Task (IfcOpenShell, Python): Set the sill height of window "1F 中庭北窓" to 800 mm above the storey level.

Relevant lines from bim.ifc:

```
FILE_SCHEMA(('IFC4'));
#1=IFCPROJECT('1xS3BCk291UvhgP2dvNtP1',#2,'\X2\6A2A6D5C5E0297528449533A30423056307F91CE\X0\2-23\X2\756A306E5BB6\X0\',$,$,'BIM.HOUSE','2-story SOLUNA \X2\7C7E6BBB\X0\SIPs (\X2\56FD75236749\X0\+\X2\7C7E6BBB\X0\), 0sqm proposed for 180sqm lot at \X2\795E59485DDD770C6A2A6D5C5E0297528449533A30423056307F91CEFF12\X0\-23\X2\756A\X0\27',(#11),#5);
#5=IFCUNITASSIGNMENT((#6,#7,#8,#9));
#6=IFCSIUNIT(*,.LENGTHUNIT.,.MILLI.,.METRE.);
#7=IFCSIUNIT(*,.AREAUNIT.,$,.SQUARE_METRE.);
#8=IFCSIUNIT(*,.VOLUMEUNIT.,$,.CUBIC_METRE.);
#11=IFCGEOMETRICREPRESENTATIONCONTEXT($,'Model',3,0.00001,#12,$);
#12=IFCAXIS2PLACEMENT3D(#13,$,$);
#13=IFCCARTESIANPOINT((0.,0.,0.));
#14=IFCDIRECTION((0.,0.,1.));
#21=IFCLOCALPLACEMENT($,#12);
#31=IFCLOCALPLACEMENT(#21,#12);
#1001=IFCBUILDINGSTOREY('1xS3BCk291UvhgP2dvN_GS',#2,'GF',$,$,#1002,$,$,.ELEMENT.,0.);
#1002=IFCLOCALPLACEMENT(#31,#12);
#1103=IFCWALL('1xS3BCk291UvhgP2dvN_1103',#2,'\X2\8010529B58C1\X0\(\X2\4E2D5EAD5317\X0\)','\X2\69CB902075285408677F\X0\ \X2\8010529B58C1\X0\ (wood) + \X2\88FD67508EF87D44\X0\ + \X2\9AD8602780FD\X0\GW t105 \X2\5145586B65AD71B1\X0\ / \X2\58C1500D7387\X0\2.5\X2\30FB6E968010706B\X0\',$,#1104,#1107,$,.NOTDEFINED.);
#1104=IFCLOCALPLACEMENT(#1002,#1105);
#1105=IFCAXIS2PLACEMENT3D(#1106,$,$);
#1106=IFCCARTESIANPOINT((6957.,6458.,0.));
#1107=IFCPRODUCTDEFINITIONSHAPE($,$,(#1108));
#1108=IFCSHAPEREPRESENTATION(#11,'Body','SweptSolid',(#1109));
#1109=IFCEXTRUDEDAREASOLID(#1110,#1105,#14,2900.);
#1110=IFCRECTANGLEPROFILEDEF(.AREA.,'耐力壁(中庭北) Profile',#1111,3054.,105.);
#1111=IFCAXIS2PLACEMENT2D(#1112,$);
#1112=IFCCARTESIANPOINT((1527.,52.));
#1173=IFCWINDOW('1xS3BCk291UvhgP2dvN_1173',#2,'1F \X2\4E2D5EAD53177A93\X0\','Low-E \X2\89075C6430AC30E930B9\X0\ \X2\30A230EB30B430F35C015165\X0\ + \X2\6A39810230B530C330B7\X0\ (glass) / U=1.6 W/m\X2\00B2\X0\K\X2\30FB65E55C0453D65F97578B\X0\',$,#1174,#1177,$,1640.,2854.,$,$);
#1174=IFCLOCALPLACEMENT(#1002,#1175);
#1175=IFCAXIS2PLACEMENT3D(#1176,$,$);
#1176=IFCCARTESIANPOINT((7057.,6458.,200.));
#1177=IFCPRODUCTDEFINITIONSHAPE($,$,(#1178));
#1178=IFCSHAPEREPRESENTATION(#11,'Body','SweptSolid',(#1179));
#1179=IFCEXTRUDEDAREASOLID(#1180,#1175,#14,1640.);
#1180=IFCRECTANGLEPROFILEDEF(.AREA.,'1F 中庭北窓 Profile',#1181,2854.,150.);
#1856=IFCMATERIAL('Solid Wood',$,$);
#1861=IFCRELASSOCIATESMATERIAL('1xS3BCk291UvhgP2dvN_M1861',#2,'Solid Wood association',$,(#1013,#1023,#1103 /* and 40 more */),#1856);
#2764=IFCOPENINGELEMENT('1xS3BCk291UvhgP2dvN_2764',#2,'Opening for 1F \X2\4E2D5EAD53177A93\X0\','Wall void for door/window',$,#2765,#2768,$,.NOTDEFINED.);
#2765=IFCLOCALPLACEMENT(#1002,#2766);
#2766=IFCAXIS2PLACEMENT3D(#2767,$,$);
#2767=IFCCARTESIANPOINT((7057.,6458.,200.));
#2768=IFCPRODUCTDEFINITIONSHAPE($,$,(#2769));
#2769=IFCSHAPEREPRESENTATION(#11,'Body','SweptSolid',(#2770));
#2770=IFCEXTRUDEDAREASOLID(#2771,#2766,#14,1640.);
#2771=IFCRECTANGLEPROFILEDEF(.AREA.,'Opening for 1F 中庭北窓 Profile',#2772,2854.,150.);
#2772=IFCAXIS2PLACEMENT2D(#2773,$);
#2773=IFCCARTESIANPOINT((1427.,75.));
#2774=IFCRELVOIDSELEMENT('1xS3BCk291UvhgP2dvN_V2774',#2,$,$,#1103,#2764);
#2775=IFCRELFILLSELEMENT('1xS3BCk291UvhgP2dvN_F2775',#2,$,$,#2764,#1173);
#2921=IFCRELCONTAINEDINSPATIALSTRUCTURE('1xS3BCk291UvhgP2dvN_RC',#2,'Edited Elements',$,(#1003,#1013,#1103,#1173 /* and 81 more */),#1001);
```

```python
import numpy as np
import ifcopenshell
import ifcopenshell.api.geometry
import ifcopenshell.geom
import ifcopenshell.util.element
import ifcopenshell.util.placement
import ifcopenshell.util.shape
import ifcopenshell.util.unit

model = ifcopenshell.open("bim.ifc")
unit_scale = ifcopenshell.util.unit.calculate_unit_scale(model)

window = model.by_guid("1xS3BCk291UvhgP2dvN_1173")
opening = window.FillsVoids[0].RelatingOpeningElement
storey = ifcopenshell.util.element.get_container(window, ifc_class="IfcBuildingStorey")
level = ifcopenshell.util.placement.get_local_placement(storey.ObjectPlacement)[2, 3]

# The opening's origin need not be at the sill, so measure its lowest point.
shape = ifcopenshell.geom.create_shape(ifcopenshell.geom.settings(), opening)
bottom = ifcopenshell.util.shape.get_shape_bottom_elevation(shape, shape.geometry) / unit_scale
dz = level + 0.8 / unit_scale - bottom

shift = np.array([0.0, 0.0, dz])
# The window is not placed relative to its opening, so move both.
for product in (opening, window):
    matrix = ifcopenshell.util.placement.get_local_placement(product.ObjectPlacement)
    matrix[:3, 3] += shift
    ifcopenshell.api.geometry.edit_object_placement(model, product=product, matrix=matrix, is_si=False)

print(f"moved by {dz * unit_scale:+.3f} m")

model.write("bim_updated.ifc")
```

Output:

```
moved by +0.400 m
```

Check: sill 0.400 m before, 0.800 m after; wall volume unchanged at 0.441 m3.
